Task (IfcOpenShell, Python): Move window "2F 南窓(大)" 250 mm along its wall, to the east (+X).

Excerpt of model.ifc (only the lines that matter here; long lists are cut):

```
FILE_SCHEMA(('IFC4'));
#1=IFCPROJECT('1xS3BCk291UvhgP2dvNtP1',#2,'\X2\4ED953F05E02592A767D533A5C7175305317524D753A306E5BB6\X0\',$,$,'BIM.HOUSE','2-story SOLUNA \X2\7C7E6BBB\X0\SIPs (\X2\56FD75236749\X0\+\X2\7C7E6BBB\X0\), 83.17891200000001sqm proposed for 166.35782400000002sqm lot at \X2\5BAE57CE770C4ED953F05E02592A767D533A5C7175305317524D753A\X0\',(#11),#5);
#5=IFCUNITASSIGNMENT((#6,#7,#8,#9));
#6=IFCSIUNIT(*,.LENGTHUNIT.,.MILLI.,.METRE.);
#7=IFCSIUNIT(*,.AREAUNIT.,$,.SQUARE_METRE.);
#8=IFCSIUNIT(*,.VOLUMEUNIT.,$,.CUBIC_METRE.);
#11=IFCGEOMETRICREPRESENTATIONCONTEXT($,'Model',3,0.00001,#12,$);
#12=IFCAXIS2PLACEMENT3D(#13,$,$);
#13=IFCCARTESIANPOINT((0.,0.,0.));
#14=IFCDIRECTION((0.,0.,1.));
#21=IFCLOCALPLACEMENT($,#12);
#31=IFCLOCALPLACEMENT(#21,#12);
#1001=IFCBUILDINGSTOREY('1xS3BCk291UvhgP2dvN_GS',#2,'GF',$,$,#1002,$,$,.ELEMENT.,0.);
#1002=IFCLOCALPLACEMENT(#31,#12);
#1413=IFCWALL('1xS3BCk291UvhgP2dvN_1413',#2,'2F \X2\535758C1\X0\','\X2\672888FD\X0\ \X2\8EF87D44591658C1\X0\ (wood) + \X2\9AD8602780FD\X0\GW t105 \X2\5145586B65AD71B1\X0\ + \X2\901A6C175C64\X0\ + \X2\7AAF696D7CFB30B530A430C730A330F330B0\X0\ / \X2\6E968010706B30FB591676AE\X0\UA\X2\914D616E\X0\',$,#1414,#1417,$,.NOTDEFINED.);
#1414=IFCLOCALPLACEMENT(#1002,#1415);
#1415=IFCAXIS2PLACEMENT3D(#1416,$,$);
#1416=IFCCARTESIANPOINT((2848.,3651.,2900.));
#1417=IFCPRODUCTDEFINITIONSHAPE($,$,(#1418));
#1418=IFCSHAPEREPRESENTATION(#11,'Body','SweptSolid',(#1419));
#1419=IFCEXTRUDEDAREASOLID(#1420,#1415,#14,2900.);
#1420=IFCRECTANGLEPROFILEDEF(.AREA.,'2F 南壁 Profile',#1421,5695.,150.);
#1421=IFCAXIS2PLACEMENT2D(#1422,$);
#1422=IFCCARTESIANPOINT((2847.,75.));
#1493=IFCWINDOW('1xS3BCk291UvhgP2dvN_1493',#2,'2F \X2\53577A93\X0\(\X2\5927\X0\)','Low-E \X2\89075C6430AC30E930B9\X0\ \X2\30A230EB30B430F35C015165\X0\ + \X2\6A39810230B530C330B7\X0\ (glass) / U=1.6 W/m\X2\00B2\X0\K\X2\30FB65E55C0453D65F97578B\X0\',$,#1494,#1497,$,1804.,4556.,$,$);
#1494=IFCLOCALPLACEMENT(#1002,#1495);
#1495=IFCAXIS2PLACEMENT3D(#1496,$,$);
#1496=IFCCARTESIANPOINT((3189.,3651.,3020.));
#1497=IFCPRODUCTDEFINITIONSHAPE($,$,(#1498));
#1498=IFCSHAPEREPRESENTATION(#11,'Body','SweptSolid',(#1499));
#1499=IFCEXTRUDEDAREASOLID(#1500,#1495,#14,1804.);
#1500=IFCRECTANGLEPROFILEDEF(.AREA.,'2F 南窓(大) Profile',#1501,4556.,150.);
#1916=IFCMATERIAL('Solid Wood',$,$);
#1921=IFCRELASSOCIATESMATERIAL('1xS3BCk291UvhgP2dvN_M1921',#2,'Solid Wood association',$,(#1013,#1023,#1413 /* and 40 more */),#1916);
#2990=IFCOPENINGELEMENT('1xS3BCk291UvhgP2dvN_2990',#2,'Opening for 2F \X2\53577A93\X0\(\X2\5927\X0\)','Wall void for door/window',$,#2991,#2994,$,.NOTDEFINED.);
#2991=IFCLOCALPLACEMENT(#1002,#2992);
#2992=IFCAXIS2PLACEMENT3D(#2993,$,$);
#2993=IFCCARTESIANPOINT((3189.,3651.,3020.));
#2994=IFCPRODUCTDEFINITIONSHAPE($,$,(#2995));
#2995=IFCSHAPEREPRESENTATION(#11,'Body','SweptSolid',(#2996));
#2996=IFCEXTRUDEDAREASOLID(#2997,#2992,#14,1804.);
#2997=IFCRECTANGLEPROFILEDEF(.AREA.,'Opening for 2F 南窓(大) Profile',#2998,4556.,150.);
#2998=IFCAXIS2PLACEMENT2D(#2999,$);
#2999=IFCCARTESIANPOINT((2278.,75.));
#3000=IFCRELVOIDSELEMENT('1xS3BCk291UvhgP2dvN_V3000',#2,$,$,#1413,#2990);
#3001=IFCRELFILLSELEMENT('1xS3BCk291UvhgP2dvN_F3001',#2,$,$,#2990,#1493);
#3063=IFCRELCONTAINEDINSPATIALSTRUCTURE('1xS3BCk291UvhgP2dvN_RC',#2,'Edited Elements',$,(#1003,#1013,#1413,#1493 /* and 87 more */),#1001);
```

```python
import ifcopenshell
import ifcopenshell.api.geometry
import ifcopenshell.util.placement
import ifcopenshell.util.unit

model = ifcopenshell.open("model.ifc")
unit_scale = ifcopenshell.util.unit.calculate_unit_scale(model)

window = model.by_guid("1xS3BCk291UvhgP2dvN_1493")
opening = window.FillsVoids[0].RelatingOpeningElement
wall = opening.VoidsElements[0].RelatingBuildingElement

wall_matrix = ifcopenshell.util.placement.get_local_placement(wall.ObjectPlacement)
shift = wall_matrix[:3, 0] * 0.25 / unit_scale
before = ifcopenshell.util.placement.get_local_placement(window.ObjectPlacement)[:3, 3].copy()

# The window is not placed relative to its opening, so move both.
for product in (opening, window):
    matrix = ifcopenshell.util.placement.get_local_placement(product.ObjectPlacement)
    matrix[:3, 3] += shift
    ifcopenshell.api.geometry.edit_object_placement(model, product=product, matrix=matrix, is_si=False)

after = ifcopenshell.util.placement.get_local_placement(window.ObjectPlacement)[:3, 3]
print("window moved by", (after - before).round(3) + 0.0)

model.write("model_updated.ifc")
```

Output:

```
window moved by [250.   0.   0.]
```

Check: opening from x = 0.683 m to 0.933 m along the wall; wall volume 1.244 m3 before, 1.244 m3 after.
